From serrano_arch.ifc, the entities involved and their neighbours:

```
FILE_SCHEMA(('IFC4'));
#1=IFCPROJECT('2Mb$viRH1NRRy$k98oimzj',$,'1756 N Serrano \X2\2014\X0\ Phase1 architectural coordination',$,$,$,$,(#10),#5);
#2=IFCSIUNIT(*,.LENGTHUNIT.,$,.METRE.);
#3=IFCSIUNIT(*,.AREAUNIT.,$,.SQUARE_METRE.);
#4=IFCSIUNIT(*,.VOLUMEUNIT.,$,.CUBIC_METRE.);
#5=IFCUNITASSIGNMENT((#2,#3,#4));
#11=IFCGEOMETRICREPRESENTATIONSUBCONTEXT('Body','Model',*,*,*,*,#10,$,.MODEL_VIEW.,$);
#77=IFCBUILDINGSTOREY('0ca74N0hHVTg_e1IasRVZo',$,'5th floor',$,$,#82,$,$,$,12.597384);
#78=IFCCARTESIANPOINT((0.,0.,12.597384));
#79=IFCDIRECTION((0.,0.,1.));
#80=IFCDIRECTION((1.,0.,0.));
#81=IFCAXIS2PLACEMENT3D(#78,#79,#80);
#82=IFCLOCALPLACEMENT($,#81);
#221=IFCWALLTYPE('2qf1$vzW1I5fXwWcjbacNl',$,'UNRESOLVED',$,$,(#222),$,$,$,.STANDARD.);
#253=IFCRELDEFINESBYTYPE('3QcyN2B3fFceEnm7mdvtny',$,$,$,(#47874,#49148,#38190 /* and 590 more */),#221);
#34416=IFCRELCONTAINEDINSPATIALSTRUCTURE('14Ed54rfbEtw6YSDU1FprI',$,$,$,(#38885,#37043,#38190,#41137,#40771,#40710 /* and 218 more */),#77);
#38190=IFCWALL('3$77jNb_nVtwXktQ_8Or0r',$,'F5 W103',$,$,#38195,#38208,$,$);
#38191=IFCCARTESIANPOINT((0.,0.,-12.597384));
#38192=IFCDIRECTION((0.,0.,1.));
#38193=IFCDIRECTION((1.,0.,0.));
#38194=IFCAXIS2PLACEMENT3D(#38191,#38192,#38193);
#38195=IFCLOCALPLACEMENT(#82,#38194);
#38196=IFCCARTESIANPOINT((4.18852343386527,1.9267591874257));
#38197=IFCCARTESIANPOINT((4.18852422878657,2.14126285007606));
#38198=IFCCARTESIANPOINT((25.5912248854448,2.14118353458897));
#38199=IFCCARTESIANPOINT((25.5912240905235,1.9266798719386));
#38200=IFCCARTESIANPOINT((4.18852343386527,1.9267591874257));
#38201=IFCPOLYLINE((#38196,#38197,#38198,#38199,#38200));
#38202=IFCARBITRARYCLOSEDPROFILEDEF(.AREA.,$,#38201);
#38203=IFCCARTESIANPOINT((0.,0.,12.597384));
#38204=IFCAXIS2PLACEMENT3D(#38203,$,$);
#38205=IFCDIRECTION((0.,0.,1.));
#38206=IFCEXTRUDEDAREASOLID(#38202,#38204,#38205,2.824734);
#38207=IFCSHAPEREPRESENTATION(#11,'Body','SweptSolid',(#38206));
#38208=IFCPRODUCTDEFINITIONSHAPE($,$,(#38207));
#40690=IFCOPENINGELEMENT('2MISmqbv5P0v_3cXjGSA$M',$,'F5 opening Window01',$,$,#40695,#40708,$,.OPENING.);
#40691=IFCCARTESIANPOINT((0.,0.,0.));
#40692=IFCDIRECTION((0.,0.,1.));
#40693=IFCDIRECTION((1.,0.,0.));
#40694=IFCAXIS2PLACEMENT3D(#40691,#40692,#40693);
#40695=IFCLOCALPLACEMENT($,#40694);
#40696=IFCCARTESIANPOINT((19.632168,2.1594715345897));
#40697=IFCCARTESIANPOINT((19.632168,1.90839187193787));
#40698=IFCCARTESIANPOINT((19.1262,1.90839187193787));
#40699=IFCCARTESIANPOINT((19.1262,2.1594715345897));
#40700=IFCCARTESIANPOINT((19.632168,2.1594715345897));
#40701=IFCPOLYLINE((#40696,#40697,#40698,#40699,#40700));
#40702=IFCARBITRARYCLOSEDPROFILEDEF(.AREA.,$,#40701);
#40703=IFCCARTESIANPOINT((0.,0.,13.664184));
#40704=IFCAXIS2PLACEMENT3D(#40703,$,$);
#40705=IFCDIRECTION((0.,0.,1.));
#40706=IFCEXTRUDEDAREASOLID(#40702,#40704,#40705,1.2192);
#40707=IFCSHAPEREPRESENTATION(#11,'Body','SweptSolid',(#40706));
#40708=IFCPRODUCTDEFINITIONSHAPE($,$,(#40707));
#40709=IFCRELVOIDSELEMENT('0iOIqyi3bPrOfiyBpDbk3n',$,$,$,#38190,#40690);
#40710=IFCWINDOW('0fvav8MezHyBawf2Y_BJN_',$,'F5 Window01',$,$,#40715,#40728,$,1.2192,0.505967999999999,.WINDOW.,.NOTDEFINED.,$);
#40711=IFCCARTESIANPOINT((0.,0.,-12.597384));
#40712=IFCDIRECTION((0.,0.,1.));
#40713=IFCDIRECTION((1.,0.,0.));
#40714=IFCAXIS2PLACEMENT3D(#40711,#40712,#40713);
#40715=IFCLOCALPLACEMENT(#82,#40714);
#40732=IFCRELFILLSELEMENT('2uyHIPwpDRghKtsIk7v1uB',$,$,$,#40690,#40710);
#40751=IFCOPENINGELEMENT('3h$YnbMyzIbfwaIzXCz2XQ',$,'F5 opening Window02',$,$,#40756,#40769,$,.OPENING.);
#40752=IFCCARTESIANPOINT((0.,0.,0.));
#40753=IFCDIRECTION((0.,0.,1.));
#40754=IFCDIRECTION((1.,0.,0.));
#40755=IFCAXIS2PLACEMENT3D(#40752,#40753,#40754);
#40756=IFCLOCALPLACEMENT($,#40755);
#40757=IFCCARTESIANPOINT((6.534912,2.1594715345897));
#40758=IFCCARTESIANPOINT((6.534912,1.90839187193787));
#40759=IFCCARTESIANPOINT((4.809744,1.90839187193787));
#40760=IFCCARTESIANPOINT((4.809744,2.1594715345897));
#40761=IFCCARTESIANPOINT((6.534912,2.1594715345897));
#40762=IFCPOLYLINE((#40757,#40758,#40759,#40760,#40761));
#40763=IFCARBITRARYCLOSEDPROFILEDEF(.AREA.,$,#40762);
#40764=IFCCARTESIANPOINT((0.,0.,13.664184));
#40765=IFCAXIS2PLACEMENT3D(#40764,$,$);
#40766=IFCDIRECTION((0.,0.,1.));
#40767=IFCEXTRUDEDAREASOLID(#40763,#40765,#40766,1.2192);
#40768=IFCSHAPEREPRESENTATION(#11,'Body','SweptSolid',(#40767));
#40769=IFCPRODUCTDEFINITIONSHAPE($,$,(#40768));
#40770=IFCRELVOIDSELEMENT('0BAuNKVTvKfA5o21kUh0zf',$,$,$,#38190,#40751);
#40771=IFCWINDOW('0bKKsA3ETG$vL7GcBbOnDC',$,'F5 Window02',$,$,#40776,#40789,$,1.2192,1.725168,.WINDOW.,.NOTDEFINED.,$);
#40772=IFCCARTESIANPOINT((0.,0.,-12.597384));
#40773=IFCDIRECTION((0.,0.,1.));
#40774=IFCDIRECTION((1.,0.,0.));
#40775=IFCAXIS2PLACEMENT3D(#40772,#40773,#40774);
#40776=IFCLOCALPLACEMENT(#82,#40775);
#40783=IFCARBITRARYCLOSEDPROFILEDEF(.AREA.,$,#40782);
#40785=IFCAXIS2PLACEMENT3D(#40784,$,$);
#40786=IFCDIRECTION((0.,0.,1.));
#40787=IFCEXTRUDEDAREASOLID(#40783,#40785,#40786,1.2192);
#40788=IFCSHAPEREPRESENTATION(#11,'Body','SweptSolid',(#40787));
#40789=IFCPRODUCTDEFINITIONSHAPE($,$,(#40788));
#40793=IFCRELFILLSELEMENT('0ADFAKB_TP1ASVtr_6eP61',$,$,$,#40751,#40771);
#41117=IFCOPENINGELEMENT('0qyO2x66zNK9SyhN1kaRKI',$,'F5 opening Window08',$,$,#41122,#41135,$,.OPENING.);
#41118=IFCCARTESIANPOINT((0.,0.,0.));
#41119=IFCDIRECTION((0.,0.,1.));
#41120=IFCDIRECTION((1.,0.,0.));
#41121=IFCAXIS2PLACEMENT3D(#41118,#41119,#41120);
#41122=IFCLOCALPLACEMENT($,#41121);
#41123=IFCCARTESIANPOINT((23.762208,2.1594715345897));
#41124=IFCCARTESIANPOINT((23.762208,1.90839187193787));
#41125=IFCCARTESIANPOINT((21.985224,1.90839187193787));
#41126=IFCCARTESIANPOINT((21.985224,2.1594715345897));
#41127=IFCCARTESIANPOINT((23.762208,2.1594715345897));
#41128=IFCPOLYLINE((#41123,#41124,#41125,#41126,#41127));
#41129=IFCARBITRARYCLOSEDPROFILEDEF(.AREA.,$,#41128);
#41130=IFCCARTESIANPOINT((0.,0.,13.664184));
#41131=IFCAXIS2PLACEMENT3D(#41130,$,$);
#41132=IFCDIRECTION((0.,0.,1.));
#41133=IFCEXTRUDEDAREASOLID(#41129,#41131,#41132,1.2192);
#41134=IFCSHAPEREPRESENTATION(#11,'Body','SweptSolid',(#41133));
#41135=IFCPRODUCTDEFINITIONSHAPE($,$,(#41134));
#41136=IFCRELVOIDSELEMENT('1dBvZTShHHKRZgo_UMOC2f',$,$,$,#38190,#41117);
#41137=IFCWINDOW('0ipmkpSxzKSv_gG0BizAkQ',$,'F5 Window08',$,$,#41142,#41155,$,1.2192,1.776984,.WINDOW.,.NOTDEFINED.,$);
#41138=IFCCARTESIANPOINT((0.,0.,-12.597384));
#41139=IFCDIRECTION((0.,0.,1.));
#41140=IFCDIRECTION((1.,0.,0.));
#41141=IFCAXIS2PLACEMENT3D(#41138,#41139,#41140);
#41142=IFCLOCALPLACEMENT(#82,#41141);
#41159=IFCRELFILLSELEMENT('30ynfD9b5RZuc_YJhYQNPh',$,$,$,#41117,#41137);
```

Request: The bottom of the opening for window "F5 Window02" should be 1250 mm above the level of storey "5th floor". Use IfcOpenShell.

```python
import numpy as np
import ifcopenshell
import ifcopenshell.api.geometry
import ifcopenshell.geom
import ifcopenshell.util.element
import ifcopenshell.util.placement
import ifcopenshell.util.shape
import ifcopenshell.util.unit

model = ifcopenshell.open("serrano_arch.ifc")
unit_scale = ifcopenshell.util.unit.calculate_unit_scale(model)

window = model.by_guid("0bKKsA3ETG$vL7GcBbOnDC")
opening = window.FillsVoids[0].RelatingOpeningElement
storey = ifcopenshell.util.element.get_container(window, ifc_class="IfcBuildingStorey")
level = ifcopenshell.util.placement.get_local_placement(storey.ObjectPlacement)[2, 3]

# The opening's origin need not be at the sill, so measure its lowest point.
shape = ifcopenshell.geom.create_shape(ifcopenshell.geom.settings(), opening)
bottom = ifcopenshell.util.shape.get_shape_bottom_elevation(shape, shape.geometry) / unit_scale
dz = level + 1.25 / unit_scale - bottom

shift = np.array([0.0, 0.0, dz])
# The window is not placed relative to its opening, so move both.
for product in (opening, window):
    matrix = ifcopenshell.util.placement.get_local_placement(product.ObjectPlacement)
    matrix[:3, 3] += shift
    ifcopenshell.api.geometry.edit_object_placement(model, product=product, matrix=matrix, is_si=False)

print(f"moved by {dz * unit_scale:+.3f} m")

model.write("serrano_arch_v2.ifc")
```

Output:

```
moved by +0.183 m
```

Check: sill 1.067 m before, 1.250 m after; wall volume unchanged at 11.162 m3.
